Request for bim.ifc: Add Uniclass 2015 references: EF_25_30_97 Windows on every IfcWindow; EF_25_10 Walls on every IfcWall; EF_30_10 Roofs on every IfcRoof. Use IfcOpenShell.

First a look at what the model holds.

```python
import ifcopenshell

model = ifcopenshell.open("bim.ifc")
print(model.schema)
print("classifications:", [c.Name for c in model.by_type("IfcClassification")])
for ifc_class in ("IfcDoor", "IfcRoof", "IfcStair", "IfcWall", "IfcWindow"):
    print(ifc_class, len(model.by_type(ifc_class)))
```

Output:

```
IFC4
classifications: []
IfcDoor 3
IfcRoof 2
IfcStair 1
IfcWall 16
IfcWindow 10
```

```python
import ifcopenshell
import ifcopenshell.api.classification

model = ifcopenshell.open("bim.ifc")

system = ifcopenshell.api.classification.add_classification(model, classification="Uniclass 2015")

codes = {
    "IfcWindow": ("EF_25_30_97", "Windows"),
    "IfcWall": ("EF_25_10", "Walls"),
    "IfcRoof": ("EF_30_10", "Roofs"),
}
for ifc_class, (code, name) in codes.items():
    products = model.by_type(ifc_class)
    ifcopenshell.api.classification.add_reference(
        model, products=products, classification=system, identification=code, name=name
    )
    print(code, len(products))

model.write("bim_edited.ifc")
```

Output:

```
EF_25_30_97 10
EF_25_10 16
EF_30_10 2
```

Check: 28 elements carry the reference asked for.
